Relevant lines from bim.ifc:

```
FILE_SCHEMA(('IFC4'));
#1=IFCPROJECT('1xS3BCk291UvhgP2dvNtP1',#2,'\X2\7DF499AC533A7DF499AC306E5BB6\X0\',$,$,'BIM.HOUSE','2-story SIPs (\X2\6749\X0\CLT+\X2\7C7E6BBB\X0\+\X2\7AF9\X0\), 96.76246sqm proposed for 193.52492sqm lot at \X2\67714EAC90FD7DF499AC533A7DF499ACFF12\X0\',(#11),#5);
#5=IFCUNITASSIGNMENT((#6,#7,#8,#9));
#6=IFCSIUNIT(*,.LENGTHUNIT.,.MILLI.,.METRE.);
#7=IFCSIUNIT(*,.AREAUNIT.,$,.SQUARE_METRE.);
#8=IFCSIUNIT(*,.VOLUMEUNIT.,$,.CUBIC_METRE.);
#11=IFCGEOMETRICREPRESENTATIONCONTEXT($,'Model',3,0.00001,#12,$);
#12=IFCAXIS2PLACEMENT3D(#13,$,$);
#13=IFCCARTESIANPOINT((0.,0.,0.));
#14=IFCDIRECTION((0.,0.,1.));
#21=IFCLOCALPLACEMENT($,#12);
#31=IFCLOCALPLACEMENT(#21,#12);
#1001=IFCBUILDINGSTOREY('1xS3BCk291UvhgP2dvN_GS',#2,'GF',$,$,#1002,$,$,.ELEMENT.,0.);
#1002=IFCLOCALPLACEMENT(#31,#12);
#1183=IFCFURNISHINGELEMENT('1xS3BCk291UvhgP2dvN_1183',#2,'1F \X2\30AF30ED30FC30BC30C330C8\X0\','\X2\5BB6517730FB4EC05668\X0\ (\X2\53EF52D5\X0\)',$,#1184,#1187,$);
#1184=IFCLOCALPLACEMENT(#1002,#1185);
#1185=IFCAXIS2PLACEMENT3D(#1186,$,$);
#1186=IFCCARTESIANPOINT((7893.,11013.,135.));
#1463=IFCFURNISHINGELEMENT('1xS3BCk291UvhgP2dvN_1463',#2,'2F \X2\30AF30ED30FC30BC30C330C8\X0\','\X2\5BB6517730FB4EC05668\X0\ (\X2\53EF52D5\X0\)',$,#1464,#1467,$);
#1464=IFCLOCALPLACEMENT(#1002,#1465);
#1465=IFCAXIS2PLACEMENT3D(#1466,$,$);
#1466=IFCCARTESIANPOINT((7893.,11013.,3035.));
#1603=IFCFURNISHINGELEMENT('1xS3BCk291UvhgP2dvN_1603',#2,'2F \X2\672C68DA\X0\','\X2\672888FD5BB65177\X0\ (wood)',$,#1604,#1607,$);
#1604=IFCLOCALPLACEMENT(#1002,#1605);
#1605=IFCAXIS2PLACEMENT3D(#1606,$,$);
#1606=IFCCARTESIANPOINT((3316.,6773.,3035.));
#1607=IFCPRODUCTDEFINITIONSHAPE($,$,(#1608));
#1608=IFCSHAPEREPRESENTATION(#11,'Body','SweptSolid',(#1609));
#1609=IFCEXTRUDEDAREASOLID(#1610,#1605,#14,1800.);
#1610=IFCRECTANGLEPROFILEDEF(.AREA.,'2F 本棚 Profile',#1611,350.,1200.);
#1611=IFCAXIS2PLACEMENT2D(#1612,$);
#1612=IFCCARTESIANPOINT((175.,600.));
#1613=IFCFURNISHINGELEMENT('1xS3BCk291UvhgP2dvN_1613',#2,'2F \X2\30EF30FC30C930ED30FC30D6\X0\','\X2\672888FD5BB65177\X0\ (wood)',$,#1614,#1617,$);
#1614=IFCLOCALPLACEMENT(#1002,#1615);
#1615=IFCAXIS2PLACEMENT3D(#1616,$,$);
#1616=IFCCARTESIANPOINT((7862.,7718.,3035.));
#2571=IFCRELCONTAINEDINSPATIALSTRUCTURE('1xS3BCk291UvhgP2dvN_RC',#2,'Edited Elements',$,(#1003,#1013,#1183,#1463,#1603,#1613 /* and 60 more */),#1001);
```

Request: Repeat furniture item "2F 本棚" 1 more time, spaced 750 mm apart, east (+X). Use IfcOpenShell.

```python
import numpy as np
import ifcopenshell
import ifcopenshell.api.geometry
import ifcopenshell.api.root
import ifcopenshell.util.element
import ifcopenshell.util.placement

model = ifcopenshell.open("bim.ifc")


def reuse_history(source, copy):
    """copy_class also copies each property set's owner history, people and application; keep the originals."""
    for rel in copy.IsDefinedBy:
        if rel.is_a("IfcRelDefinesByProperties") and (history := rel.RelatingPropertyDefinition.OwnerHistory):
            rel.RelatingPropertyDefinition.OwnerHistory = source.OwnerHistory
            ifcopenshell.util.element.remove_deep2(model, history)


source = model.by_guid("1xS3BCk291UvhgP2dvN_1603")
base = ifcopenshell.util.placement.get_local_placement(source.ObjectPlacement)
step = np.array([1.0, 0.0, 0.0]) * 750.0

for i in range(1, 2):
    copy = ifcopenshell.api.root.copy_class(model, product=source)
    copy.Representation = ifcopenshell.util.element.copy_deep(
        model, source.Representation, exclude=["IfcGeometricRepresentationContext", "IfcRepresentationMap"]
    )
    reuse_history(source, copy)
    matrix = base.copy()
    matrix[:3, 3] += i * step
    print("added at", matrix[:3, 3].round(3) + 0.0)
    ifcopenshell.api.geometry.edit_object_placement(model, product=copy, matrix=matrix, is_si=False)

model.write("bim_rev.ifc")
```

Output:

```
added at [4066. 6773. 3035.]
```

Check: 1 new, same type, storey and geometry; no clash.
